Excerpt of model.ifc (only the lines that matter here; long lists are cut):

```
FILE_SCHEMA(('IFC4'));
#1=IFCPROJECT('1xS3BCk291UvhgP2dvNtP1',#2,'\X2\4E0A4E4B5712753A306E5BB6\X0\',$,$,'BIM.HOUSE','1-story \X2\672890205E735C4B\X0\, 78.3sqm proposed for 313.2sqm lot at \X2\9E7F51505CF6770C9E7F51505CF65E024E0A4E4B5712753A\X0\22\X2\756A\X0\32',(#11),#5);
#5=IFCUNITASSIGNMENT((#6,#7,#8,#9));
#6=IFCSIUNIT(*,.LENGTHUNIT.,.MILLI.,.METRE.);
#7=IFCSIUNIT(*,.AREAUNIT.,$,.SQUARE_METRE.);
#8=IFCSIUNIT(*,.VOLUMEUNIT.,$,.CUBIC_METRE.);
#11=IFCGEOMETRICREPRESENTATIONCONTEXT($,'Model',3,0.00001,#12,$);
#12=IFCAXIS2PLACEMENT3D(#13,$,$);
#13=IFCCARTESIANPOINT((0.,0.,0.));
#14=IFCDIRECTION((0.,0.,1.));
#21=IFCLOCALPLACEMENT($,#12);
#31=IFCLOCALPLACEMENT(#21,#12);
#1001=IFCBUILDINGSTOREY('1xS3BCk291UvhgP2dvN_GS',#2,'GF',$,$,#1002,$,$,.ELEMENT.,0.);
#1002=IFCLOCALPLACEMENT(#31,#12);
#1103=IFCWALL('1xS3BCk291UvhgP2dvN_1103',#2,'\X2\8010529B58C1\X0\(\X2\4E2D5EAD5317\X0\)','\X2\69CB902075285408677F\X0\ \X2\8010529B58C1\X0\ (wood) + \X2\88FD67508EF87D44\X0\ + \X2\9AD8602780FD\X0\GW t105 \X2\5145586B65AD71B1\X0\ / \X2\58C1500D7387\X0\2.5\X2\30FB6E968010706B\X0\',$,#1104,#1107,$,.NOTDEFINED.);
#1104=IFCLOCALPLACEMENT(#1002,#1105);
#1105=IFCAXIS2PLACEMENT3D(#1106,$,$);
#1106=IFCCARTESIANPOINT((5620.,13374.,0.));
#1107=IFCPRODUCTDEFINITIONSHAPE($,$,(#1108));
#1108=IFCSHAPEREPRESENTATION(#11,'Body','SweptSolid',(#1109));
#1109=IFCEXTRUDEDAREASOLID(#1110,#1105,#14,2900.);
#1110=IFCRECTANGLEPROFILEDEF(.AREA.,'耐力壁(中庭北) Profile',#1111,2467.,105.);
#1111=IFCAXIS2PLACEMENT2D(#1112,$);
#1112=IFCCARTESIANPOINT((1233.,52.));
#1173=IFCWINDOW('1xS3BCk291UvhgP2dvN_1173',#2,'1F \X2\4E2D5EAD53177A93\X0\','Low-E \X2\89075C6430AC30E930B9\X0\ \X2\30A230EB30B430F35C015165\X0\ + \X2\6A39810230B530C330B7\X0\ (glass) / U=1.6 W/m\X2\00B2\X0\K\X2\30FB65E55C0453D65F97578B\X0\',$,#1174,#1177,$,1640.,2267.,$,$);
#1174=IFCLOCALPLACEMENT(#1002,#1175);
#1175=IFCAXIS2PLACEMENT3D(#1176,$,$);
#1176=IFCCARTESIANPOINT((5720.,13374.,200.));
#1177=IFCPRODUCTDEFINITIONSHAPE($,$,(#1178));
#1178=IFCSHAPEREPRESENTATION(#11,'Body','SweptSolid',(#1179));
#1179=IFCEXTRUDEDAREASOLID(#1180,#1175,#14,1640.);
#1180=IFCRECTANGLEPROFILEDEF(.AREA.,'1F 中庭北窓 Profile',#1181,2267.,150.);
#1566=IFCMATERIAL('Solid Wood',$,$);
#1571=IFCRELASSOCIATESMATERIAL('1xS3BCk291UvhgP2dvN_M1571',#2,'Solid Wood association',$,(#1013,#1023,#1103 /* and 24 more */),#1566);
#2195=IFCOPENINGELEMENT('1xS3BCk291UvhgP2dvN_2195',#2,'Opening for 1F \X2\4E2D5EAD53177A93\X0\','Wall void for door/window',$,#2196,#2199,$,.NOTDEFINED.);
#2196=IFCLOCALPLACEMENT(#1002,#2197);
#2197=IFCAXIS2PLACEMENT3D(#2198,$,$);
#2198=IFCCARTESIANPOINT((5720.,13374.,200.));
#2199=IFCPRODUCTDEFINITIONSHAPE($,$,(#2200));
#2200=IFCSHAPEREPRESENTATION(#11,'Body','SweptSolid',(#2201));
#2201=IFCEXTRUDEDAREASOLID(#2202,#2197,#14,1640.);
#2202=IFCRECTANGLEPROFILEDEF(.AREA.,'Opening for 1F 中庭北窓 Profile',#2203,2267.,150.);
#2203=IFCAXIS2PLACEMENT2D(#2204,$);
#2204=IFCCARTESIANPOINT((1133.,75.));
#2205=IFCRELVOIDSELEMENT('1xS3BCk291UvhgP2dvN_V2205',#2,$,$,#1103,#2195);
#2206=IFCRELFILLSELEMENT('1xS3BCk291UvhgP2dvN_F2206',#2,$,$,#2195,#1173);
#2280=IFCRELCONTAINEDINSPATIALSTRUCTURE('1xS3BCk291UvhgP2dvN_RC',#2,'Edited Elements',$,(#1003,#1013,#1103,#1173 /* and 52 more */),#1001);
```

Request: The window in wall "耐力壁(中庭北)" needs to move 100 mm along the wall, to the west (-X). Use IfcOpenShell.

```python
import ifcopenshell
import ifcopenshell.api.geometry
import ifcopenshell.util.placement

model = ifcopenshell.open("model.ifc")

window = model.by_id(1173)
opening = window.FillsVoids[0].RelatingOpeningElement
wall = opening.VoidsElements[0].RelatingBuildingElement

wall_matrix = ifcopenshell.util.placement.get_local_placement(wall.ObjectPlacement)
shift = wall_matrix[:3, 0] * -100.0
before = ifcopenshell.util.placement.get_local_placement(window.ObjectPlacement)[:3, 3].copy()

# The window is not placed relative to its opening, so move both.
for product in (opening, window):
    matrix = ifcopenshell.util.placement.get_local_placement(product.ObjectPlacement)
    matrix[:3, 3] += shift
    ifcopenshell.api.geometry.edit_object_placement(model, product=product, matrix=matrix, is_si=False)

after = ifcopenshell.util.placement.get_local_placement(window.ObjectPlacement)[:3, 3]
print("window moved by", (after - before).round(3) + 0.0)

model.write("model_updated.ifc")
```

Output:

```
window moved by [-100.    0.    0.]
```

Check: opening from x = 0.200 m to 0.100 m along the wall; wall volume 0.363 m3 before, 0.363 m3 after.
